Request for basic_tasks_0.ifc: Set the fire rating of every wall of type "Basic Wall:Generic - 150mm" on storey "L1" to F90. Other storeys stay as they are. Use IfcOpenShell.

First a look at what the model holds.

```python
import ifcopenshell
import ifcopenshell.util.element

model = ifcopenshell.open("basic_tasks_0.ifc")
print(model.schema)
storey = next(s for s in model.by_type("IfcBuildingStorey") if s.Name == "L1")
walls = [e for e in ifcopenshell.util.element.get_decomposition(storey) if e.is_a("IfcWall")]
seen = {}
for e in walls:
    element_type = ifcopenshell.util.element.get_type(e)
    key = (element_type.Name if element_type != e and element_type else None, ifcopenshell.util.element.get_pset(e, "Pset_WallCommon", "FireRating"))
    seen[key] = seen.get(key, 0) + 1
for (name, value), count in sorted(seen.items(), key=str):
    print(count, "x", name, "|", value)
```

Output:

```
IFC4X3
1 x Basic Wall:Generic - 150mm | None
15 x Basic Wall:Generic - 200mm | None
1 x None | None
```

```python
import ifcopenshell
import ifcopenshell.api.pset
import ifcopenshell.util.element

model = ifcopenshell.open("basic_tasks_0.ifc")

storey = next(s for s in model.by_type("IfcBuildingStorey") if s.Name == "L1")
walls = [e for e in ifcopenshell.util.element.get_decomposition(storey) if e.is_a("IfcWall")]

count = 0
for e in walls:
    element_type = ifcopenshell.util.element.get_type(e)
    if element_type in (None, e) or element_type.Name != "Basic Wall:Generic - 150mm":
        continue
    # add_pset returns the element's existing set when there is one.
    pset = ifcopenshell.api.pset.add_pset(model, product=e, name="Pset_WallCommon")
    ifcopenshell.api.pset.edit_pset(model, pset=pset, properties={"FireRating": "F90"})
    count += 1

print(count, "walls updated")

model.write("basic_tasks_0_v2.ifc")
```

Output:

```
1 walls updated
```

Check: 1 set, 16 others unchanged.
